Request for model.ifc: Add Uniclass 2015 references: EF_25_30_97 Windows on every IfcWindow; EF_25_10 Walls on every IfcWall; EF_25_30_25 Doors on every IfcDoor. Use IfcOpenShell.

First a look at what the model holds.

```python
import ifcopenshell

model = ifcopenshell.open("model.ifc")
print(model.schema)
print("classifications:", [c.Name for c in model.by_type("IfcClassification")])
for ifc_class in ("IfcDoor", "IfcRoof", "IfcStair", "IfcWall", "IfcWindow"):
    print(ifc_class, len(model.by_type(ifc_class)))
```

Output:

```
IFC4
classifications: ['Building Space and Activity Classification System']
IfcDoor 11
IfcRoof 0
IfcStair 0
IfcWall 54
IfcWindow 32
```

```python
import ifcopenshell
import ifcopenshell.api.classification

model = ifcopenshell.open("model.ifc")

system = ifcopenshell.api.classification.add_classification(model, classification="Uniclass 2015")

codes = {
    "IfcWindow": ("EF_25_30_97", "Windows"),
    "IfcWall": ("EF_25_10", "Walls"),
    "IfcDoor": ("EF_25_30_25", "Doors"),
}
for ifc_class, (code, name) in codes.items():
    products = model.by_type(ifc_class)
    ifcopenshell.api.classification.add_reference(
        model, products=products, classification=system, identification=code, name=name
    )
    print(code, len(products))

model.write("model-out.ifc")
```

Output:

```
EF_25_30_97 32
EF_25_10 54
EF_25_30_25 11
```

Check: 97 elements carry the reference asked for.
